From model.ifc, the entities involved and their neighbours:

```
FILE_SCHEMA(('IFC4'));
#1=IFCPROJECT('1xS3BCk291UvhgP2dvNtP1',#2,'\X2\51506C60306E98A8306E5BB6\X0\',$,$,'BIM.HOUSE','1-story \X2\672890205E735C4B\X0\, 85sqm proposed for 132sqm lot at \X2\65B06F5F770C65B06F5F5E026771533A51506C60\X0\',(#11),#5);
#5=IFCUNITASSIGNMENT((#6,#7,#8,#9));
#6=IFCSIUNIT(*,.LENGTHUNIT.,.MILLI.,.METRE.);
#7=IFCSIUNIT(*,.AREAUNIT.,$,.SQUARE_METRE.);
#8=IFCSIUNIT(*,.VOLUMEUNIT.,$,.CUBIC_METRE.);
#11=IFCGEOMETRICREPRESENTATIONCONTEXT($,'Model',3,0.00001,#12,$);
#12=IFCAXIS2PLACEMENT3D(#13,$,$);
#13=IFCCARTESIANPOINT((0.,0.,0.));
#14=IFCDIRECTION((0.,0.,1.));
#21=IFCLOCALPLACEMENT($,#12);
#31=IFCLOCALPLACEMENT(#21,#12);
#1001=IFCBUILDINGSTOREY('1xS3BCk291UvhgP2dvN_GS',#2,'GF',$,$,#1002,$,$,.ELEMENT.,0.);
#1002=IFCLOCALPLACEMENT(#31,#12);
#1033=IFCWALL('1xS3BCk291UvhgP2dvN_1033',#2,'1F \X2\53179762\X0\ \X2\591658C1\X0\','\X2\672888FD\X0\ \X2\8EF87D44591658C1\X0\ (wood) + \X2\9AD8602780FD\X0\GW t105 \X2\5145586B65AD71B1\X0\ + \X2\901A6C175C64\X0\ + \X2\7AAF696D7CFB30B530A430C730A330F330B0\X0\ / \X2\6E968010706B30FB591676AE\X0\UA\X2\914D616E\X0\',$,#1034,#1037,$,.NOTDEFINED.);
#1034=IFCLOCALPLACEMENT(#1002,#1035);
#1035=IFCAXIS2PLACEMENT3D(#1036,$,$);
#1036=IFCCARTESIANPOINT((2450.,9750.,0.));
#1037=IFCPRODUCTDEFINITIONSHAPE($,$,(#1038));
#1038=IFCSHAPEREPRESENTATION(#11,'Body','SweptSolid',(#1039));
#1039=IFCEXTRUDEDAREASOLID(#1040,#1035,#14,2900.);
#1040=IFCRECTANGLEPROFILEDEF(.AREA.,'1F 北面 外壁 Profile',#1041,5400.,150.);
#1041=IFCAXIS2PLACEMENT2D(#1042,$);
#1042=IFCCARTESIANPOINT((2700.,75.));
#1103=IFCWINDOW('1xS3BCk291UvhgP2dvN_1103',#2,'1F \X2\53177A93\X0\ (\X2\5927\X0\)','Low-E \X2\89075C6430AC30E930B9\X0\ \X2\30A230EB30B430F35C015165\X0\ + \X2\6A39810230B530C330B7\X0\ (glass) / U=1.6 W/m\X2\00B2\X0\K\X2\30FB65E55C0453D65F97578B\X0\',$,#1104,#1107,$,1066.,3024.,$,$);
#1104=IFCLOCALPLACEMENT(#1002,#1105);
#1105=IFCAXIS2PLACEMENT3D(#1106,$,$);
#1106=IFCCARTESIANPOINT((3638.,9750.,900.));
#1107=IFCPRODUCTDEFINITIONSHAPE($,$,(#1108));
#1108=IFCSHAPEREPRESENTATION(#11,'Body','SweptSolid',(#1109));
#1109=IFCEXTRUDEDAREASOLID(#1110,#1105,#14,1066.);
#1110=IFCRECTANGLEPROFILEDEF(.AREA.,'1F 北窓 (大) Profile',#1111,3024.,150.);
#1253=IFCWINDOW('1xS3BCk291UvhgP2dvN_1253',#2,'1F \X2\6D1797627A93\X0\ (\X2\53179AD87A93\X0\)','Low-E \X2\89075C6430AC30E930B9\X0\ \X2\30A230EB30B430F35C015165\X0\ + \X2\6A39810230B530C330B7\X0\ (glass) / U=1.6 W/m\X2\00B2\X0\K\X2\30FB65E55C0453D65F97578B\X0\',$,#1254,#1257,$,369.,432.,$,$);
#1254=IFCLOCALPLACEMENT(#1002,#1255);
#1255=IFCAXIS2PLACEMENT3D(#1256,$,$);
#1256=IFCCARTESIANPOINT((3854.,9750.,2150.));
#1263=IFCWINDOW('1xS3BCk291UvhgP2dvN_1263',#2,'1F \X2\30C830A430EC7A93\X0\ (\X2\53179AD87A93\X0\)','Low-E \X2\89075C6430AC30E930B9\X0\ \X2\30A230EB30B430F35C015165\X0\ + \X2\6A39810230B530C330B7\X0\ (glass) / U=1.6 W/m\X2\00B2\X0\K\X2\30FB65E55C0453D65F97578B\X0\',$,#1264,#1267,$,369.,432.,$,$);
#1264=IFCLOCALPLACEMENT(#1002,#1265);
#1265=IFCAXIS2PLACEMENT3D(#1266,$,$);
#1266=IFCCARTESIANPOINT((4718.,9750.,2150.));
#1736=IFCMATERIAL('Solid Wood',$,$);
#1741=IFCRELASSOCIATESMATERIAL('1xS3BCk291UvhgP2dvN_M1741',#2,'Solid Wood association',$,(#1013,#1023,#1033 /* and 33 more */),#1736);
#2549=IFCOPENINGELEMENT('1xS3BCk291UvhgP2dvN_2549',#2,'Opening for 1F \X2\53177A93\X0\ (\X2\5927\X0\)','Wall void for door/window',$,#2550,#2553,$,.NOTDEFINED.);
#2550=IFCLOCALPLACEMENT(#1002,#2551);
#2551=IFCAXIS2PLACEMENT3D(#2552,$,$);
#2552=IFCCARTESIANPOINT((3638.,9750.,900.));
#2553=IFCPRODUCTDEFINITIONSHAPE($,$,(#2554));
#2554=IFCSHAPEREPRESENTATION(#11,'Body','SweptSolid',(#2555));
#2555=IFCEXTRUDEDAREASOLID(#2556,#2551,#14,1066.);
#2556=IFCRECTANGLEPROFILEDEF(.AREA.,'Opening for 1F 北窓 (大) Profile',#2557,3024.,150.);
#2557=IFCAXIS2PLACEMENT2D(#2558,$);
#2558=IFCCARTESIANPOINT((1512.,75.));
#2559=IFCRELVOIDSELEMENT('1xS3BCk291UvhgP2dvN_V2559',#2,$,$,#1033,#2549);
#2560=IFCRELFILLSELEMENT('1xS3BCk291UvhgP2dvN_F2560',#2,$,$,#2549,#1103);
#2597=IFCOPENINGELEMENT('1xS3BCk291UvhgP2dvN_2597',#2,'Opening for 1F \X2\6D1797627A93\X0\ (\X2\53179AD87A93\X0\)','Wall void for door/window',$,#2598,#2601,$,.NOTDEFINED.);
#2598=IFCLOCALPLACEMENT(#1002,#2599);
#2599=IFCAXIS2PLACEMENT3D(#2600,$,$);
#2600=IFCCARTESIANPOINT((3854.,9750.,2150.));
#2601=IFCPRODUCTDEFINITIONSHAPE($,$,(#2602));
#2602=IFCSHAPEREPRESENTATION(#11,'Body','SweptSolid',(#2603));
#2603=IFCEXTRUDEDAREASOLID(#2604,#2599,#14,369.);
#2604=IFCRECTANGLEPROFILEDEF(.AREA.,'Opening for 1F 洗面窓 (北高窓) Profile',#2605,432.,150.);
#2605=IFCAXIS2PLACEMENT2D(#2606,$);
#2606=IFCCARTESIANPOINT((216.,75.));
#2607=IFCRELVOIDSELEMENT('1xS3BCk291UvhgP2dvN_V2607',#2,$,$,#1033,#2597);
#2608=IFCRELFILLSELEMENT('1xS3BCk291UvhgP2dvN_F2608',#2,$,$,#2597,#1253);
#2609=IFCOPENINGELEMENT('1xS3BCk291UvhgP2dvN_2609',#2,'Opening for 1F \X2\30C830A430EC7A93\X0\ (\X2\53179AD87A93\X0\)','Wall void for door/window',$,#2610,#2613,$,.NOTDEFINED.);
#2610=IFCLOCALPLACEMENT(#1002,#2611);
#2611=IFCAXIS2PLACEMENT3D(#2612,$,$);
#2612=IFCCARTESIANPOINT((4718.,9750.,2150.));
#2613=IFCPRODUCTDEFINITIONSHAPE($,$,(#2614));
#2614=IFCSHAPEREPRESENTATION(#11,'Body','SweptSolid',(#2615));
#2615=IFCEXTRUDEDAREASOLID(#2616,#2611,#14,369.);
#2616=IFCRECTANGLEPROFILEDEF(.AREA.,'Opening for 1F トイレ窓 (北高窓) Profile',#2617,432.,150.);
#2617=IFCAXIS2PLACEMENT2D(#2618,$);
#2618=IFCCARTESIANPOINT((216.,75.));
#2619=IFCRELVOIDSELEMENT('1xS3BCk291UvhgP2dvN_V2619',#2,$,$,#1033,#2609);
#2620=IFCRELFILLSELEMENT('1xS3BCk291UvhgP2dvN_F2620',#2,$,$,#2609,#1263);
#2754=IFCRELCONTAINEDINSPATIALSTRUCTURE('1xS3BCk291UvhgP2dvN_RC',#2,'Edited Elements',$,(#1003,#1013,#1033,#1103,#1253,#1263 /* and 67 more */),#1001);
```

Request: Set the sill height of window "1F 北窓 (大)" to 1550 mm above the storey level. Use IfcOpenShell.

```python
import numpy as np
import ifcopenshell
import ifcopenshell.api.geometry
import ifcopenshell.geom
import ifcopenshell.util.element
import ifcopenshell.util.placement
import ifcopenshell.util.shape
import ifcopenshell.util.unit

model = ifcopenshell.open("model.ifc")
unit_scale = ifcopenshell.util.unit.calculate_unit_scale(model)

window = model.by_guid("1xS3BCk291UvhgP2dvN_1103")
opening = window.FillsVoids[0].RelatingOpeningElement
storey = ifcopenshell.util.element.get_container(window, ifc_class="IfcBuildingStorey")
level = ifcopenshell.util.placement.get_local_placement(storey.ObjectPlacement)[2, 3]

# The opening's origin need not be at the sill, so measure its lowest point.
shape = ifcopenshell.geom.create_shape(ifcopenshell.geom.settings(), opening)
bottom = ifcopenshell.util.shape.get_shape_bottom_elevation(shape, shape.geometry) / unit_scale
dz = level + 1550.0 - bottom

shift = np.array([0.0, 0.0, dz])
# The window is not placed relative to its opening, so move both.
for product in (opening, window):
    matrix = ifcopenshell.util.placement.get_local_placement(product.ObjectPlacement)
    matrix[:3, 3] += shift
    ifcopenshell.api.geometry.edit_object_placement(model, product=product, matrix=matrix, is_si=False)

print(f"moved by {dz * unit_scale:+.3f} m")

model.write("model_rev.ifc")
```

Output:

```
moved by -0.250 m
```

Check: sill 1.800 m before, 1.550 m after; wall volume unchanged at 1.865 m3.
